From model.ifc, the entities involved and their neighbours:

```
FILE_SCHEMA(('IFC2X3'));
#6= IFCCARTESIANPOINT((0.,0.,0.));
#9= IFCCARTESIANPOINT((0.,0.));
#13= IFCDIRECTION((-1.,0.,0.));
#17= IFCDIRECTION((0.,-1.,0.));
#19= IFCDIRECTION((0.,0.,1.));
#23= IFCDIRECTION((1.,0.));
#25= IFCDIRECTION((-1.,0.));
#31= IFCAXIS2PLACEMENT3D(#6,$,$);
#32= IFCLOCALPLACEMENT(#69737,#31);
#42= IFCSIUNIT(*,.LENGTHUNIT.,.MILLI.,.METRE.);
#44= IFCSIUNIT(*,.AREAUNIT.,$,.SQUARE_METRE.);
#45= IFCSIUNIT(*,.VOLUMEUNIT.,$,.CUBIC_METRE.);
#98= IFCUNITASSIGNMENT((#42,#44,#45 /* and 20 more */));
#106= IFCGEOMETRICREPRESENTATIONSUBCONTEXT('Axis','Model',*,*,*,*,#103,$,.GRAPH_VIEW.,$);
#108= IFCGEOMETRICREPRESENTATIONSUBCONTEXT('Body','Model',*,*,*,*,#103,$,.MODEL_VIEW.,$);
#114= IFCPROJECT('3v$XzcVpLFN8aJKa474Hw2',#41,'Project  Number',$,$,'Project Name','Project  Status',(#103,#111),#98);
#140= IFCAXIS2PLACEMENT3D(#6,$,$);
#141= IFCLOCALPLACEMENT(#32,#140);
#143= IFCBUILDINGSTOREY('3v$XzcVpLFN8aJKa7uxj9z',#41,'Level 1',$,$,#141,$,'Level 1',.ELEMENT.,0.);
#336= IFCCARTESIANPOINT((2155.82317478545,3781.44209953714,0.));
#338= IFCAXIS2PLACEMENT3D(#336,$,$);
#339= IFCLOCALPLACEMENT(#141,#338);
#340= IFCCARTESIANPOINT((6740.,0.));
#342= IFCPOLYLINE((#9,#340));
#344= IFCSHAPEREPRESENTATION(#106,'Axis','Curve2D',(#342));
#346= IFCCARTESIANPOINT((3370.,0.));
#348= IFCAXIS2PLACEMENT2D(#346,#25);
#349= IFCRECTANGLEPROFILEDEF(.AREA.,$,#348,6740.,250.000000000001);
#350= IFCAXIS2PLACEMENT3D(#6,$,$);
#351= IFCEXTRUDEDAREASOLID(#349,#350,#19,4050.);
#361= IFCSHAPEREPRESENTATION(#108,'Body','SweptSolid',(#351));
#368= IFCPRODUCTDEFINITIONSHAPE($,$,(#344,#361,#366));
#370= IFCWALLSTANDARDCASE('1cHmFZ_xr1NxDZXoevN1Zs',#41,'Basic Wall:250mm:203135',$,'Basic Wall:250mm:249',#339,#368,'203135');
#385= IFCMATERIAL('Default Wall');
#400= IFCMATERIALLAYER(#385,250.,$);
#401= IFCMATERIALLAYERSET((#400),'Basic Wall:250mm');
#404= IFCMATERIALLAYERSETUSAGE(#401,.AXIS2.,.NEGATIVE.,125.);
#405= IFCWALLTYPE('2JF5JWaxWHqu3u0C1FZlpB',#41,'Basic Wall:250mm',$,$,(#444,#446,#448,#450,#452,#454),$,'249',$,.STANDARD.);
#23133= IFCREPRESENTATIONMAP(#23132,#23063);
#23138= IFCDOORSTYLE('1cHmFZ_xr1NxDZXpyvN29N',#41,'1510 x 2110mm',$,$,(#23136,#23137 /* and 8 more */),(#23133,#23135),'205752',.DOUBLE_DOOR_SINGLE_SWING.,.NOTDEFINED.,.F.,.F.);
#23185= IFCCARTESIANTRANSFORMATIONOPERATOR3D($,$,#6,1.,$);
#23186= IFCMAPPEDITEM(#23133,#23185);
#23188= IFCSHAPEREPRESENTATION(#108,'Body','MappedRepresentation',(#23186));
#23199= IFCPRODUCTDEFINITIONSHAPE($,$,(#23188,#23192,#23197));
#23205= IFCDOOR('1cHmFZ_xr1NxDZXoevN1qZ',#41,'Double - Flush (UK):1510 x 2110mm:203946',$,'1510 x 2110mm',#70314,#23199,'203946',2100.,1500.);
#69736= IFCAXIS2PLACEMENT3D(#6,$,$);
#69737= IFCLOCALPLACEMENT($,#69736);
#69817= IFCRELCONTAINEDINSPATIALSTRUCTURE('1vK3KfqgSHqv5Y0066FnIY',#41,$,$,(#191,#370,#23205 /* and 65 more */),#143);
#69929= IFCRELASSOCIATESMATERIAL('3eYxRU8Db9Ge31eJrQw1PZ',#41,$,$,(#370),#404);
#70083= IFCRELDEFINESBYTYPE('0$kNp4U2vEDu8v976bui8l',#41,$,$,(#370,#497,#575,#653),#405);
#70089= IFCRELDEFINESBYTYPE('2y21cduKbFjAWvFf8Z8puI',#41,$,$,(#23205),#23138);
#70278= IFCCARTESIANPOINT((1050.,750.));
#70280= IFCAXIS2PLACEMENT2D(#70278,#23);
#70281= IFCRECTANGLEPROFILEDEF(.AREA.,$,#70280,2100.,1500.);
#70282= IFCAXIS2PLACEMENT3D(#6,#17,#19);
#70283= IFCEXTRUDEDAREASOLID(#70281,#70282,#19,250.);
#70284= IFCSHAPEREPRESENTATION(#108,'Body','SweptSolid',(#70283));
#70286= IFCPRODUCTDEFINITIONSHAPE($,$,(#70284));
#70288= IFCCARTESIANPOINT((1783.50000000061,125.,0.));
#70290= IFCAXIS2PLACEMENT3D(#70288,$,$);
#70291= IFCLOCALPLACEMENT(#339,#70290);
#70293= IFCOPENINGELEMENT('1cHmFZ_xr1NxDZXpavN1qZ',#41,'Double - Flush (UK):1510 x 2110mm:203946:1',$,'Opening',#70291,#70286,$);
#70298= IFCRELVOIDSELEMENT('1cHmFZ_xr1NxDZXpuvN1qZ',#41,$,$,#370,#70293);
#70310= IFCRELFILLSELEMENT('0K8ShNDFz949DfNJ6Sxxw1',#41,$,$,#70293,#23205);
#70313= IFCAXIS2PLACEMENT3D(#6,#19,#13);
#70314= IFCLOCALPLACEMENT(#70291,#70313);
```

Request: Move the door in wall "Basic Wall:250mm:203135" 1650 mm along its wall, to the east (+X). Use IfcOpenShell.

```python
import ifcopenshell
import ifcopenshell.api.geometry
import ifcopenshell.util.placement
import ifcopenshell.util.unit

model = ifcopenshell.open("model.ifc")
unit_scale = ifcopenshell.util.unit.calculate_unit_scale(model)

door = model.by_guid("1cHmFZ_xr1NxDZXoevN1qZ")
opening = door.FillsVoids[0].RelatingOpeningElement
wall = opening.VoidsElements[0].RelatingBuildingElement

wall_matrix = ifcopenshell.util.placement.get_local_placement(wall.ObjectPlacement)
shift = wall_matrix[:3, 0] * 1.65 / unit_scale
before = ifcopenshell.util.placement.get_local_placement(door.ObjectPlacement)[:3, 3].copy()

# The door is placed relative to its opening, so it follows when the opening moves.
matrix = ifcopenshell.util.placement.get_local_placement(opening.ObjectPlacement)
matrix[:3, 3] += shift
ifcopenshell.api.geometry.edit_object_placement(
    model, product=opening, matrix=matrix, is_si=False, should_transform_children=True
)

after = ifcopenshell.util.placement.get_local_placement(door.ObjectPlacement)[:3, 3]
print("door moved by", (after - before).round(3) + 0.0)

model.write("model_edited.ifc")
```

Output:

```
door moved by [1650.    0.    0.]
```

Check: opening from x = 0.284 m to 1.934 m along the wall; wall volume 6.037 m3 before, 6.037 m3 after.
